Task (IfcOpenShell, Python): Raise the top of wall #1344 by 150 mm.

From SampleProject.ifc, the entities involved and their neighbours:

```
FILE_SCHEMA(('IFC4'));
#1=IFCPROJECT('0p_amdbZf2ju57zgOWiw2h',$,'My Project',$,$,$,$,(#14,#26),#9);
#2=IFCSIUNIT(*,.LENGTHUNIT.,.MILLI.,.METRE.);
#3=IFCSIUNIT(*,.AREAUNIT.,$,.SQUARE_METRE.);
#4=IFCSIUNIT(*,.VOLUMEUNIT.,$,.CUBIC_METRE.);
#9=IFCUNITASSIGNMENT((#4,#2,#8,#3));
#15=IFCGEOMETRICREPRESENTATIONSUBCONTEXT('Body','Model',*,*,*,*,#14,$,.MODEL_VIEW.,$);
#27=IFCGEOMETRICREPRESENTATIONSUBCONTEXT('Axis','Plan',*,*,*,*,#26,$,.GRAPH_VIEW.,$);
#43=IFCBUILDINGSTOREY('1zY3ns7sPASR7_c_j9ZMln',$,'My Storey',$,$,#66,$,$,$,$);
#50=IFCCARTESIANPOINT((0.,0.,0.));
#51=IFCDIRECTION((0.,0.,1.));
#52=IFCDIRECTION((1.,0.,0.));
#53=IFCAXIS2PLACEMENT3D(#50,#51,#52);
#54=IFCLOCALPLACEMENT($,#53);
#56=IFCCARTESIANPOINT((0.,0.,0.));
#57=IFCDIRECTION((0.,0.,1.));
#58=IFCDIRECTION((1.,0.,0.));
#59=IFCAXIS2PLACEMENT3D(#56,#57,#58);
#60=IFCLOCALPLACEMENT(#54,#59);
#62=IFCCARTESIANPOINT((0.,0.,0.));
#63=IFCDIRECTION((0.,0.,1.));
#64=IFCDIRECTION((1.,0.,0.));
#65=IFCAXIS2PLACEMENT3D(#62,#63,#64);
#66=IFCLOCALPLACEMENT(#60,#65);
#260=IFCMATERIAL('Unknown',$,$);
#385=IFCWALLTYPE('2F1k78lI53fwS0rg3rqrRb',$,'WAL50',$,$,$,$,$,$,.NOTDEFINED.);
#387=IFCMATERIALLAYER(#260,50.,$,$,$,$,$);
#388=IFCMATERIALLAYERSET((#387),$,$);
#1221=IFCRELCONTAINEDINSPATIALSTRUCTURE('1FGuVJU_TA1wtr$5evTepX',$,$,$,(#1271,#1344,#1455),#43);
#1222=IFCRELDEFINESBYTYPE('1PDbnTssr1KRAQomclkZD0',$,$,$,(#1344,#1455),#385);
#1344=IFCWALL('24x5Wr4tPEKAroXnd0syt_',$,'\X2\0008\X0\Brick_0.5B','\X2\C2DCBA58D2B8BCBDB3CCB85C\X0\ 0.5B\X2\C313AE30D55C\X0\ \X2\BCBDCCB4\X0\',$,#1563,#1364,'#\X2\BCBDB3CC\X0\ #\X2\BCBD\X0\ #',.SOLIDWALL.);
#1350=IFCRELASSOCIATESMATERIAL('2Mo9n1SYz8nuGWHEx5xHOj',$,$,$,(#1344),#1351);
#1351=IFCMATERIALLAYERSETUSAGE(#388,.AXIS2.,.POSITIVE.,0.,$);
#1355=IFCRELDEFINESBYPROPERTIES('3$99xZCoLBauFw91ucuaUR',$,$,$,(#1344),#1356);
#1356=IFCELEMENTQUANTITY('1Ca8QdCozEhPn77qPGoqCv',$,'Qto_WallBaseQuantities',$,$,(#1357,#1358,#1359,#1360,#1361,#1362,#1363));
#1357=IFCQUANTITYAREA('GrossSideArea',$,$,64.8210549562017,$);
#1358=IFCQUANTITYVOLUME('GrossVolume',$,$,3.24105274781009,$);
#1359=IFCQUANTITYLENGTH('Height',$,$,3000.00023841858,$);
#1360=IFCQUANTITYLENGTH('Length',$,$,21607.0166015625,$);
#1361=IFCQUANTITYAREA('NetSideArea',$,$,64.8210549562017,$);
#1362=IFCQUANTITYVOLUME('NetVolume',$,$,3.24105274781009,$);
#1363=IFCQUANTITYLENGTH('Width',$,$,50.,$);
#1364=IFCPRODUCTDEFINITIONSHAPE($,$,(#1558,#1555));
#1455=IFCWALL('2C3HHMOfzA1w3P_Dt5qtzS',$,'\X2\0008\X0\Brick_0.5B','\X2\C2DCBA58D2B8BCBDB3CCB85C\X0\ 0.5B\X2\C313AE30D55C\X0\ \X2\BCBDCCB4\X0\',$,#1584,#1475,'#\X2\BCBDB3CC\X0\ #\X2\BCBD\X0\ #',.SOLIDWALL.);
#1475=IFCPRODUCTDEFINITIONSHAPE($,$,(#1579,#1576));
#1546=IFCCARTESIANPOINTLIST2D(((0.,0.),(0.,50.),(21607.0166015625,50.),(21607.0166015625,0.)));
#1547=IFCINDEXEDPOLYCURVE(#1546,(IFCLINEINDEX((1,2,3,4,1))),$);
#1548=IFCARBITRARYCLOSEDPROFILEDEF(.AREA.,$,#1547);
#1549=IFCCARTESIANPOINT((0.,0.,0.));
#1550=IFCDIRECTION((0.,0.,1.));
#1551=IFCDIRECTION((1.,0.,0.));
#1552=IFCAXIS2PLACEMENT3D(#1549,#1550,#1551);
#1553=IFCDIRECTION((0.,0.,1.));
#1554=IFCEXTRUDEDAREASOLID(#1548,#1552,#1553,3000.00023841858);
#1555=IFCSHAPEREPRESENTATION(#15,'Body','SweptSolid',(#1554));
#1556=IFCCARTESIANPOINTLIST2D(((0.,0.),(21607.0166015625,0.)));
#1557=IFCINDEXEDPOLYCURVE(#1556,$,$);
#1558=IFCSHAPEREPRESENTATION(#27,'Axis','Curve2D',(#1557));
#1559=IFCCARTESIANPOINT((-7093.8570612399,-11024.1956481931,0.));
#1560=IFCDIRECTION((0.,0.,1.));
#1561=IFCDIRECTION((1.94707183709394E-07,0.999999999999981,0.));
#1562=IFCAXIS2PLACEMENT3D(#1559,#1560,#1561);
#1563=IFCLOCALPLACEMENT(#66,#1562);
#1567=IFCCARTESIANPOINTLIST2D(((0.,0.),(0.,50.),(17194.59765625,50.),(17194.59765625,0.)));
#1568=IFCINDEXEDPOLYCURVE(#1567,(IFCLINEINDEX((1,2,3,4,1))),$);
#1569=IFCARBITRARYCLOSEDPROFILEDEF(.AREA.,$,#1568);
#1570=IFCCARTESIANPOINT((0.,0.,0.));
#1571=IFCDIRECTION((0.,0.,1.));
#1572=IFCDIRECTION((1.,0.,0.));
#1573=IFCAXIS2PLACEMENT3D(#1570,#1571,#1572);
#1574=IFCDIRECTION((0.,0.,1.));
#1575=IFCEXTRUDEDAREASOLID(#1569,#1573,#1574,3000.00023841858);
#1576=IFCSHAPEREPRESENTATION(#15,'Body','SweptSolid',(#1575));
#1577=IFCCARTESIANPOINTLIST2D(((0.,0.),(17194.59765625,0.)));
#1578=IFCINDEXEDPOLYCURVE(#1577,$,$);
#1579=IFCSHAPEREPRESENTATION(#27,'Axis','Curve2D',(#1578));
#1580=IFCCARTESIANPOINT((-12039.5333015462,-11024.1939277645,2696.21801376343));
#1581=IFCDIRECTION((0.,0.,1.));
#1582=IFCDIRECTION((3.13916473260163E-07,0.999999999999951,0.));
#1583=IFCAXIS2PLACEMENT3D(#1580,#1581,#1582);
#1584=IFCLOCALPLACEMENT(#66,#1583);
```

```python
import ifcopenshell
import ifcopenshell.api.pset
import ifcopenshell.geom
import ifcopenshell.util.element
import ifcopenshell.util.representation
import ifcopenshell.util.shape
import ifcopenshell.util.unit

model = ifcopenshell.open("SampleProject.ifc")
unit_scale = ifcopenshell.util.unit.calculate_unit_scale(model)
area_scale = ifcopenshell.util.unit.calculate_unit_scale(model, "AREAUNIT")
volume_scale = ifcopenshell.util.unit.calculate_unit_scale(model, "VOLUMEUNIT")
settings = ifcopenshell.geom.settings()


def volume(element):
    """Net volume in cubic metres, openings subtracted."""
    shape = ifcopenshell.geom.create_shape(settings, element)
    return ifcopenshell.util.shape.get_volume(shape.geometry)


wall = model.by_id(1344)
before = volume(wall)

body = ifcopenshell.util.representation.get_representation(wall, "Model", "Body")
solid = body.Items[0]
old_height = solid.Depth
solid.Depth += 150.0
after = volume(wall)
thickness = 0.05  # wall thickness in metres

# Update the stored height, areas and volumes.
qto = model.by_id(ifcopenshell.util.element.get_pset(wall, "Qto_WallBaseQuantities", should_inherit=False)["id"])
ifcopenshell.api.pset.edit_qto(model, qto=qto, properties={
    "GrossSideArea": ifcopenshell.util.element.get_pset(wall, "Qto_WallBaseQuantities", "GrossSideArea") * solid.Depth / old_height,
    "GrossVolume": ifcopenshell.util.element.get_pset(wall, "Qto_WallBaseQuantities", "GrossVolume") * solid.Depth / old_height,
    "Height": solid.Depth,
    "NetSideArea": after / thickness / area_scale,
    "NetVolume": after / volume_scale,
})

print(f"height {old_height:g} -> {solid.Depth:g}, volume {before:.3f} -> {after:.3f} m3")

model.write("SampleProject-out.ifc")
```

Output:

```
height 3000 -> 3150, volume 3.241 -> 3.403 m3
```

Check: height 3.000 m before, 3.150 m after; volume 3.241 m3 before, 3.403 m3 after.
